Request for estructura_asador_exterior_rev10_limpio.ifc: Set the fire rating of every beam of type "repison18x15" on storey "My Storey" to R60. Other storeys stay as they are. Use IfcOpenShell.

First a look at what the model holds.

```python
import ifcopenshell
import ifcopenshell.util.element

model = ifcopenshell.open("estructura_asador_exterior_rev10_limpio.ifc")
print(model.schema)
storey = next(s for s in model.by_type("IfcBuildingStorey") if s.Name == "My Storey")
beams = [e for e in ifcopenshell.util.element.get_decomposition(storey) if e.is_a("IfcBeam")]
seen = {}
for e in beams:
    element_type = ifcopenshell.util.element.get_type(e)
    key = (element_type.Name if element_type != e and element_type else None, ifcopenshell.util.element.get_pset(e, "Pset_BeamCommon", "FireRating"))
    seen[key] = seen.get(key, 0) + 1
for (name, value), count in sorted(seen.items(), key=str):
    print(count, "x", name, "|", value)
```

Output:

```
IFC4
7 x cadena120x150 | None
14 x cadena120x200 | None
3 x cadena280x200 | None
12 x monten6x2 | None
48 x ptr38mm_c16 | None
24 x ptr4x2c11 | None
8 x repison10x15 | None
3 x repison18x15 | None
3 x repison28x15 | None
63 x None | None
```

```python
import ifcopenshell
import ifcopenshell.api.pset
import ifcopenshell.util.element

model = ifcopenshell.open("estructura_asador_exterior_rev10_limpio.ifc")

storey = next(s for s in model.by_type("IfcBuildingStorey") if s.Name == "My Storey")
beams = [e for e in ifcopenshell.util.element.get_decomposition(storey) if e.is_a("IfcBeam")]

count = 0
for e in beams:
    element_type = ifcopenshell.util.element.get_type(e)
    if element_type in (None, e) or element_type.Name != "repison18x15":
        continue
    # add_pset returns the element's existing set when there is one.
    pset = ifcopenshell.api.pset.add_pset(model, product=e, name="Pset_BeamCommon")
    ifcopenshell.api.pset.edit_pset(model, pset=pset, properties={"FireRating": "R60"})
    count += 1

print(count, "beams updated")

model.write("estructura_asador_exterior_rev10_limpio_edited.ifc")
```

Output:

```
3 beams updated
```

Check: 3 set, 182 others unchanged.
